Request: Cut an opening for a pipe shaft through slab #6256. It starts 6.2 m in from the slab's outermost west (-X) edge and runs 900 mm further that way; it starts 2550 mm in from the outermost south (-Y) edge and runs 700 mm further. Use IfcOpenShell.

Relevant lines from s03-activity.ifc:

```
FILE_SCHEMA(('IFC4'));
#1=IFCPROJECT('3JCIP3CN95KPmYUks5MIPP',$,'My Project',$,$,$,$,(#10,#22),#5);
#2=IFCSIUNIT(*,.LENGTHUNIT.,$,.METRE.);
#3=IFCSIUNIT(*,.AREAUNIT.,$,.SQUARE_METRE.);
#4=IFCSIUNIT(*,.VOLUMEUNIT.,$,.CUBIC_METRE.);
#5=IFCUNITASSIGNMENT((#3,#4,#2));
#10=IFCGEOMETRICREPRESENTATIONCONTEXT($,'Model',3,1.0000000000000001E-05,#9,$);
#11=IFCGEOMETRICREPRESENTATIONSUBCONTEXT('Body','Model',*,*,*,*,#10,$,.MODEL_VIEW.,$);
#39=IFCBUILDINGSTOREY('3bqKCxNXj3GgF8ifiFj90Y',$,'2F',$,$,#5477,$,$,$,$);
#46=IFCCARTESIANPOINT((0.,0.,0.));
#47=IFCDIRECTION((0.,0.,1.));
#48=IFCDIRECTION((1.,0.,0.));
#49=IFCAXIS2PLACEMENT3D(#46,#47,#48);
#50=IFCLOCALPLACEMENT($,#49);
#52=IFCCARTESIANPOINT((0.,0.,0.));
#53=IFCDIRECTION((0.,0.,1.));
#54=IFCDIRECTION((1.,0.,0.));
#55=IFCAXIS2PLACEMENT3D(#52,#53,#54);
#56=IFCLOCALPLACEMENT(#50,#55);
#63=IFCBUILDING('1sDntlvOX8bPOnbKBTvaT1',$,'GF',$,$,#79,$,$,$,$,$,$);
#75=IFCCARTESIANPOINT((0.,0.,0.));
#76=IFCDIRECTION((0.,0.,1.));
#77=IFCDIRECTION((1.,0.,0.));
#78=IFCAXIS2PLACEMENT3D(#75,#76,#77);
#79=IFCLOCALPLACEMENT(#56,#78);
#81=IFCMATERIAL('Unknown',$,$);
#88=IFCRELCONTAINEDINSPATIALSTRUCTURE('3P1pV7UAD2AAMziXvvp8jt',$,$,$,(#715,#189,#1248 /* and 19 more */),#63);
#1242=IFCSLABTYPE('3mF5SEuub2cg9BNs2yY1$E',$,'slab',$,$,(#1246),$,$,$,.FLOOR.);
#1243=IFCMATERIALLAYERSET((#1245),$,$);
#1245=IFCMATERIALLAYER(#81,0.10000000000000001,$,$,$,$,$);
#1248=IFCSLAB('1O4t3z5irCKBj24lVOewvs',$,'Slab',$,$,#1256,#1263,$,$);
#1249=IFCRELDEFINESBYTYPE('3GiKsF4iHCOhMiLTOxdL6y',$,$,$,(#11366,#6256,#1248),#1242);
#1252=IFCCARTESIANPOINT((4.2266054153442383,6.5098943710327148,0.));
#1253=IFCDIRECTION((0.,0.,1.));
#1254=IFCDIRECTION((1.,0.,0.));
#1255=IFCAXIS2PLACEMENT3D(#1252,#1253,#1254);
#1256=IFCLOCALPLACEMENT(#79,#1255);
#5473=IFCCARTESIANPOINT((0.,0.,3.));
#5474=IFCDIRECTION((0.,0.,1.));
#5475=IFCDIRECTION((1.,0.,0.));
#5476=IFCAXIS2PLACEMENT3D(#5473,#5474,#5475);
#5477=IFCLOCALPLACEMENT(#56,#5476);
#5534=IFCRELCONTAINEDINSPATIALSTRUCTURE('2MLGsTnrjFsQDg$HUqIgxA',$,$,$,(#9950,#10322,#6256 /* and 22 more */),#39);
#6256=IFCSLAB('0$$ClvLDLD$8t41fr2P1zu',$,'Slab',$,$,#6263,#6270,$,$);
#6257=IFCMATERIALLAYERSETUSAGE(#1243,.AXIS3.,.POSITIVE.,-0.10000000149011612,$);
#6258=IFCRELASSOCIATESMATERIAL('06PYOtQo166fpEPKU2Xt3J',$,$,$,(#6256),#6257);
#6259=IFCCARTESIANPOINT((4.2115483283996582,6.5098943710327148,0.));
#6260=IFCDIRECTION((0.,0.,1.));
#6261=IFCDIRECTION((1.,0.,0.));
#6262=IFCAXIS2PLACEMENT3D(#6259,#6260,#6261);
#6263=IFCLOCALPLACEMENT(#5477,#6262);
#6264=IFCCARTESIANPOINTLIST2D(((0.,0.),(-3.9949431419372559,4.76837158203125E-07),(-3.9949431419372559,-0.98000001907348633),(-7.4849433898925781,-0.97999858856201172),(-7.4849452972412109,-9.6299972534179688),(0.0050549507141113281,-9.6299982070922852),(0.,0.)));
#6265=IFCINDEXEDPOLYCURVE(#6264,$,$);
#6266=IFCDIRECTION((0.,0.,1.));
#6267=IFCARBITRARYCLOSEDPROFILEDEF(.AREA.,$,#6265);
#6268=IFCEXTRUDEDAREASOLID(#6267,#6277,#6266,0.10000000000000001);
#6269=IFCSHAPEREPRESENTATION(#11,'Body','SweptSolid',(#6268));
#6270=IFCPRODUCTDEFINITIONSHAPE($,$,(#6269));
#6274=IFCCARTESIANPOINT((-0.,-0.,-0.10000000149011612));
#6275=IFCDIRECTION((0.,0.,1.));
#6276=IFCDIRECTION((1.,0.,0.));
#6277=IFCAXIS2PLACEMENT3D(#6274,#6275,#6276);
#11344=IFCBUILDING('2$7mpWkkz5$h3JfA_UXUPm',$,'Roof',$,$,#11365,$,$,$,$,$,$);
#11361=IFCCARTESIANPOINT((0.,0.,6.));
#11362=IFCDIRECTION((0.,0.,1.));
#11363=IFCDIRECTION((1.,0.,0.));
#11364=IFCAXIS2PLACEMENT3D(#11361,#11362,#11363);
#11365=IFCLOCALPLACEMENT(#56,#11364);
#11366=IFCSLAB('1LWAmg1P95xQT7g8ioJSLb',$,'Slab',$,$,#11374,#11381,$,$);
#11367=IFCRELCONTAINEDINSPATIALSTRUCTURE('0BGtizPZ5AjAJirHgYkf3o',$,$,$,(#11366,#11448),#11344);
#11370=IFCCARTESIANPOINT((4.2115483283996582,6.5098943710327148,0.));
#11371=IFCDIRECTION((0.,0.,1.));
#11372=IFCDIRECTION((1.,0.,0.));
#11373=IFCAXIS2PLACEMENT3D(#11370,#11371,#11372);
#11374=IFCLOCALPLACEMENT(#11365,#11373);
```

```python
import numpy as np
import ifcopenshell
import ifcopenshell.api.feature
import ifcopenshell.api.geometry
import ifcopenshell.api.root
import ifcopenshell.geom
import ifcopenshell.util.placement
import ifcopenshell.util.representation
import ifcopenshell.util.shape
import ifcopenshell.util.unit

model = ifcopenshell.open("s03-activity.ifc")
unit_scale = ifcopenshell.util.unit.calculate_unit_scale(model)
settings = ifcopenshell.geom.settings()


def volume(element):
    """Net volume in cubic metres, openings subtracted."""
    shape = ifcopenshell.geom.create_shape(settings, element)
    return ifcopenshell.util.shape.get_volume(shape.geometry)


slab = model.by_id(6256)
before = volume(slab)

# Extent in the slab's own axes, in metres. The edges named are its -X and -Y sides.
slab_shape = ifcopenshell.geom.create_shape(settings, slab)
vertices = ifcopenshell.util.shape.get_vertices(slab_shape.geometry)
x_min, y_min, bottom = vertices.min(axis=0)
top = vertices[:, 2].max()

opening = ifcopenshell.api.root.create_entity(model, ifc_class="IfcOpeningElement", name="Pipe shaft opening", predefined_type="OPENING")
context = ifcopenshell.util.representation.get_context(model, "Model", "Body", "MODEL_VIEW")
width, depth = 0.9, 0.7
outline = [(0.0, 0.0), (width, 0.0), (width, depth), (0.0, depth), (0.0, 0.0)]
# Overshoot both faces by 50 mm so the cut is clean.
shape = ifcopenshell.api.geometry.add_slab_representation(
    model, context=context, depth=top - bottom + 0.1, polyline=outline
)
ifcopenshell.api.geometry.assign_representation(model, product=opening, representation=shape)

matrix = ifcopenshell.util.placement.get_local_placement(slab.ObjectPlacement)
matrix[:, 3] = matrix @ np.append(np.array([x_min + 6.2, y_min + 2.55, bottom - 0.05]) / unit_scale, 1.0)
ifcopenshell.api.geometry.edit_object_placement(model, product=opening, matrix=matrix, is_si=False)
ifcopenshell.api.feature.add_feature(model, feature=opening, element=slab)

after = volume(slab)

print(f"slab volume {before:.3f} -> {after:.3f} m3")

model.write("s03-activity_updated.ifc")
```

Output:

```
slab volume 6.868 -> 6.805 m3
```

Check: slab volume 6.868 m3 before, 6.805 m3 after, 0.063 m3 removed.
